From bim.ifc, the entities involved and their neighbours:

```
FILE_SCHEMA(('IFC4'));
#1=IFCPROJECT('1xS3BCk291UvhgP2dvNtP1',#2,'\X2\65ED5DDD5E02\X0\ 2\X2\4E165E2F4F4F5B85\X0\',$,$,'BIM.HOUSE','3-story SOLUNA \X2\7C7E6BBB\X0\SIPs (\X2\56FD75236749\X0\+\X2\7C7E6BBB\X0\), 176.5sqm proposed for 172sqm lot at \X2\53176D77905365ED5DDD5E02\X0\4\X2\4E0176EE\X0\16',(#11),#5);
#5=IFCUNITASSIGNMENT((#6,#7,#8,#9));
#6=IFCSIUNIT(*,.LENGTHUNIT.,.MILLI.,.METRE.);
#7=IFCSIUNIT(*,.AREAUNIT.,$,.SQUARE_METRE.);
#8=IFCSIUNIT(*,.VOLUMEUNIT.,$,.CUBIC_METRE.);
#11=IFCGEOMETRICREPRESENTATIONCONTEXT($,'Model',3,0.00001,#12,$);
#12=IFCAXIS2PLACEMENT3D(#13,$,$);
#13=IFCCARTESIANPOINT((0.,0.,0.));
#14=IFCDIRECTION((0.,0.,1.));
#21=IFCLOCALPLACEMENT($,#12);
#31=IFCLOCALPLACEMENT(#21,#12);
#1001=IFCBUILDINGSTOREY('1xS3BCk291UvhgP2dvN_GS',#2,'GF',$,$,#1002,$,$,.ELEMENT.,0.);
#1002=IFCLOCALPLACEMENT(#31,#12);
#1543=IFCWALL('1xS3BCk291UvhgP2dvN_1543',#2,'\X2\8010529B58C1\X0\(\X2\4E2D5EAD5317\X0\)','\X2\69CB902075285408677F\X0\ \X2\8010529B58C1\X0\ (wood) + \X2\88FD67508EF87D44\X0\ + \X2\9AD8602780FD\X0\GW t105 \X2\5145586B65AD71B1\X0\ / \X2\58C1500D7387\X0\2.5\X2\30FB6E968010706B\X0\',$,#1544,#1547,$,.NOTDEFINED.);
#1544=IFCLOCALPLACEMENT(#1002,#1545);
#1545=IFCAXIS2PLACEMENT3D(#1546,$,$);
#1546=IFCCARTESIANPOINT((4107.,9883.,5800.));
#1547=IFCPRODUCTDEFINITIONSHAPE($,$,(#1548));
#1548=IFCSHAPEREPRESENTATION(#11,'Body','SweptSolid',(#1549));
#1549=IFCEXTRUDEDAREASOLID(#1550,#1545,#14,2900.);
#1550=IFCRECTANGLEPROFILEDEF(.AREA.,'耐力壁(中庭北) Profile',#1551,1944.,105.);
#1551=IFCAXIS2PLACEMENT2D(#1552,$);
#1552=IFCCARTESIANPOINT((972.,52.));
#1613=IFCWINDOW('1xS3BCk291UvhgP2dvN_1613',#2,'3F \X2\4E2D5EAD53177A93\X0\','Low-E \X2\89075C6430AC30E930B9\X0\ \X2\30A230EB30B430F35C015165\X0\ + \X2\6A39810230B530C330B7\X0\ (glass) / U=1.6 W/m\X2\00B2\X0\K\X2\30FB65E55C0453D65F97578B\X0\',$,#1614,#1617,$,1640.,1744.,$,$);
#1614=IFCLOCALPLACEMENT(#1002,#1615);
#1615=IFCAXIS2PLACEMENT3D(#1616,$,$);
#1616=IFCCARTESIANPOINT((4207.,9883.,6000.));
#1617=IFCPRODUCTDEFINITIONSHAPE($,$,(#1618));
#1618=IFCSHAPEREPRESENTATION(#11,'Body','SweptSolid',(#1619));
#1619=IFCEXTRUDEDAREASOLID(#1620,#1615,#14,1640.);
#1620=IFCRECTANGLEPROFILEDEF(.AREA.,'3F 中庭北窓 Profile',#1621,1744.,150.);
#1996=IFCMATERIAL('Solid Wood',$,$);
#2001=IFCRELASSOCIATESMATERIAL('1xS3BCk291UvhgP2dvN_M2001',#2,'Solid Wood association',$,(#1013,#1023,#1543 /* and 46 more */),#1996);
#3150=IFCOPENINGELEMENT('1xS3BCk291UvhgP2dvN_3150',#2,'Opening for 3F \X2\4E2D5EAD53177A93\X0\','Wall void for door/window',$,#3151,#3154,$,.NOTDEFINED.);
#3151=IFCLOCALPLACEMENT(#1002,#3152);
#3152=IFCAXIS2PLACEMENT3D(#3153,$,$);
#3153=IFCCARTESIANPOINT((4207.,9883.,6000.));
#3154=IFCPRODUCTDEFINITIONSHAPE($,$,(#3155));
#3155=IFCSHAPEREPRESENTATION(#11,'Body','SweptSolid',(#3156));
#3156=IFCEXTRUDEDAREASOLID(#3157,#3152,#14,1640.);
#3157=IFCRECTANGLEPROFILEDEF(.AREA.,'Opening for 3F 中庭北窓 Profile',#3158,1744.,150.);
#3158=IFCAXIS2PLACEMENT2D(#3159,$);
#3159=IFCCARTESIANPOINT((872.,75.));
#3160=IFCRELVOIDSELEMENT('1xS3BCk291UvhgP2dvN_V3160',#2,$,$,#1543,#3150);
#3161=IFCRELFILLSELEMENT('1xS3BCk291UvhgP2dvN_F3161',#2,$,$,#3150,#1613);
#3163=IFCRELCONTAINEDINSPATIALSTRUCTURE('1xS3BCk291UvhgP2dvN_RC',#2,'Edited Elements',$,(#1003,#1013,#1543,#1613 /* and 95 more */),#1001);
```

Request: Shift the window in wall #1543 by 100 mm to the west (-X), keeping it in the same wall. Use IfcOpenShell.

```python
import ifcopenshell
import ifcopenshell.api.geometry
import ifcopenshell.util.placement

model = ifcopenshell.open("bim.ifc")

window = model.by_guid("1xS3BCk291UvhgP2dvN_1613")
opening = window.FillsVoids[0].RelatingOpeningElement
wall = opening.VoidsElements[0].RelatingBuildingElement

wall_matrix = ifcopenshell.util.placement.get_local_placement(wall.ObjectPlacement)
shift = wall_matrix[:3, 0] * -100.0
before = ifcopenshell.util.placement.get_local_placement(window.ObjectPlacement)[:3, 3].copy()

# The window is not placed relative to its opening, so move both.
for product in (opening, window):
    matrix = ifcopenshell.util.placement.get_local_placement(product.ObjectPlacement)
    matrix[:3, 3] += shift
    ifcopenshell.api.geometry.edit_object_placement(model, product=product, matrix=matrix, is_si=False)

after = ifcopenshell.util.placement.get_local_placement(window.ObjectPlacement)[:3, 3]
print("window moved by", (after - before).round(3) + 0.0)

model.write("bim_updated.ifc")
```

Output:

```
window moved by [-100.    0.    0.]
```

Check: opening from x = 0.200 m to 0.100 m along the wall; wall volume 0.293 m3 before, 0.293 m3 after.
